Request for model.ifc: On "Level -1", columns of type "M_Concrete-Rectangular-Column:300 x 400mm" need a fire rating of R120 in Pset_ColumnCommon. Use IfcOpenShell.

First a look at what the model holds.

```python
import ifcopenshell
import ifcopenshell.util.element

model = ifcopenshell.open("model.ifc")
print(model.schema)
storey = next(s for s in model.by_type("IfcBuildingStorey") if s.Name == "Level -1")
columns = [e for e in ifcopenshell.util.element.get_decomposition(storey) if e.is_a("IfcColumn")]
seen = {}
for e in columns:
    element_type = ifcopenshell.util.element.get_type(e)
    key = (element_type.Name if element_type != e and element_type else None, ifcopenshell.util.element.get_pset(e, "Pset_ColumnCommon", "FireRating"))
    seen[key] = seen.get(key, 0) + 1
for (name, value), count in sorted(seen.items(), key=str):
    print(count, "x", name, "|", value)
```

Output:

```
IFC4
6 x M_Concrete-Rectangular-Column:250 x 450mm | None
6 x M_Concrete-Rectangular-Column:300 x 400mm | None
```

```python
import ifcopenshell
import ifcopenshell.api.pset
import ifcopenshell.util.element

model = ifcopenshell.open("model.ifc")

storey = next(s for s in model.by_type("IfcBuildingStorey") if s.Name == "Level -1")
columns = [e for e in ifcopenshell.util.element.get_decomposition(storey) if e.is_a("IfcColumn")]

count = 0
for e in columns:
    element_type = ifcopenshell.util.element.get_type(e)
    if element_type in (None, e) or element_type.Name != "M_Concrete-Rectangular-Column:300 x 400mm":
        continue
    # add_pset returns the element's existing set when there is one.
    pset = ifcopenshell.api.pset.add_pset(model, product=e, name="Pset_ColumnCommon")
    ifcopenshell.api.pset.edit_pset(model, pset=pset, properties={"FireRating": "R120"})
    count += 1

print(count, "columns updated")

model.write("model_updated.ifc")
```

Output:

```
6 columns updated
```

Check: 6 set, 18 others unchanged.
